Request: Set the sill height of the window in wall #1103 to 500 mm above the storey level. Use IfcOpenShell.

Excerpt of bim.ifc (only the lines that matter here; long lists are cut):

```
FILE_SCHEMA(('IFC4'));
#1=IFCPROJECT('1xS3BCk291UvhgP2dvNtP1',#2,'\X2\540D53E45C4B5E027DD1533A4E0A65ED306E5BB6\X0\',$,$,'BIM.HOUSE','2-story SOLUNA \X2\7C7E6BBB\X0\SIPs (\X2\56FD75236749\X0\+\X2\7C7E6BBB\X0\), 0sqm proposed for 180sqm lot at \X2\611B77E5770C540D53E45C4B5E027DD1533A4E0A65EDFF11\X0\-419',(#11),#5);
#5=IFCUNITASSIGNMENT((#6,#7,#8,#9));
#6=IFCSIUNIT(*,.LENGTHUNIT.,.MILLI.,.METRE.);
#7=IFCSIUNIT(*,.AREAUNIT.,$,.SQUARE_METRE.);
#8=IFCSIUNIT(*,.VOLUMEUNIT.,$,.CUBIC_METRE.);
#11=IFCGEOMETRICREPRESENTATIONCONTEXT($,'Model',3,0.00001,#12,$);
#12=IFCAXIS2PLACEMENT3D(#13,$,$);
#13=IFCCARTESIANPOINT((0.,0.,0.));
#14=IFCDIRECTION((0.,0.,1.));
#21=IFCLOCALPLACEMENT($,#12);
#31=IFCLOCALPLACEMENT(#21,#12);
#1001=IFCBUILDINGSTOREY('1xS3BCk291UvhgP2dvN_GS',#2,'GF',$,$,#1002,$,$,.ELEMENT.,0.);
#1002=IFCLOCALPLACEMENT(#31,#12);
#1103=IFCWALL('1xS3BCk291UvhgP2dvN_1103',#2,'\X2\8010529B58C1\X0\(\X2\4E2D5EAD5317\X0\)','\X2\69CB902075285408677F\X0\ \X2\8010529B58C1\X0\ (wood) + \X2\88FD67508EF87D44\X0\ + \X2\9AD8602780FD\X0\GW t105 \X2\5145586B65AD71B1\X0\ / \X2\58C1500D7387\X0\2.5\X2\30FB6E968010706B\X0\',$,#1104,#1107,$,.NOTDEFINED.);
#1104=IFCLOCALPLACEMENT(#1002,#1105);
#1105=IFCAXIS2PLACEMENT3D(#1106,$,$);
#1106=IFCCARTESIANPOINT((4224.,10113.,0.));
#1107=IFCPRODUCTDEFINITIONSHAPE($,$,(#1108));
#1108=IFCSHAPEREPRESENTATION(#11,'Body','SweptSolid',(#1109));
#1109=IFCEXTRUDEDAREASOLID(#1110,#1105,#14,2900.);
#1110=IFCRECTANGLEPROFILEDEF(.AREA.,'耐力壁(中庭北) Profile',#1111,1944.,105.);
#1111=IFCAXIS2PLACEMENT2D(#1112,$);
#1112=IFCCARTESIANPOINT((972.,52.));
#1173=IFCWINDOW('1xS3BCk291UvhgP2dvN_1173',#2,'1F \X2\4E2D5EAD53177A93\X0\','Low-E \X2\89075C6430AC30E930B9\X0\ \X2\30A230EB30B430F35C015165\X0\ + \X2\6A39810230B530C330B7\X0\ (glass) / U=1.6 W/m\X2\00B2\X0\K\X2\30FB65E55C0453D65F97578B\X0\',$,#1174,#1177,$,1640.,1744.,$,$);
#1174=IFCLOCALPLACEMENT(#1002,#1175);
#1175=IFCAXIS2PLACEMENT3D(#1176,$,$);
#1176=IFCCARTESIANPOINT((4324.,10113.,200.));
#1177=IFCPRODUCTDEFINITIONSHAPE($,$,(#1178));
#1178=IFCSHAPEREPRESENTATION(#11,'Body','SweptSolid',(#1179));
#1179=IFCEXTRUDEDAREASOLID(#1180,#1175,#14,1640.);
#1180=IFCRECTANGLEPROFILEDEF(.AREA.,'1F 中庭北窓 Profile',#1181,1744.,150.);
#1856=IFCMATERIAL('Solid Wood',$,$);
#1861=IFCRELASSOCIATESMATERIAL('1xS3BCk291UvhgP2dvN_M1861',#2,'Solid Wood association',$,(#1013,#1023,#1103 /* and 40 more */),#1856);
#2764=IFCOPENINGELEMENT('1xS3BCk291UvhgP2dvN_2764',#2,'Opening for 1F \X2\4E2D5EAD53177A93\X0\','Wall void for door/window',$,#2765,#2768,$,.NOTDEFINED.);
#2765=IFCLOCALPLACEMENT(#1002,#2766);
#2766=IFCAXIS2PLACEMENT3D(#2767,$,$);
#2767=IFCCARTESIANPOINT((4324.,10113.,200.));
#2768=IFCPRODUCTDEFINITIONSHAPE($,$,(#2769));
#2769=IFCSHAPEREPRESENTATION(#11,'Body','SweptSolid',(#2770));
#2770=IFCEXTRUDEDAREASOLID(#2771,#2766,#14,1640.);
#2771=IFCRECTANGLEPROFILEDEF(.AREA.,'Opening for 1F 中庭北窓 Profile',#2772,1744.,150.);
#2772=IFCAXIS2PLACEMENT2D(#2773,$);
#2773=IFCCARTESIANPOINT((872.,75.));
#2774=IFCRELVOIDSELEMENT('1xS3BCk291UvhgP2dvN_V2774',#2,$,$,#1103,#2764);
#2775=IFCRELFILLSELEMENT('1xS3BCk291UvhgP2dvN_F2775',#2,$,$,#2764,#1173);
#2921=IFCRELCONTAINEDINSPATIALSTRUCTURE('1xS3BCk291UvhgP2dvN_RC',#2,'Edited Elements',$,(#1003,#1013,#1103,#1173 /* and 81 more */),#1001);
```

```python
import numpy as np
import ifcopenshell
import ifcopenshell.api.geometry
import ifcopenshell.geom
import ifcopenshell.util.element
import ifcopenshell.util.placement
import ifcopenshell.util.shape
import ifcopenshell.util.unit

model = ifcopenshell.open("bim.ifc")
unit_scale = ifcopenshell.util.unit.calculate_unit_scale(model)

window = model.by_guid("1xS3BCk291UvhgP2dvN_1173")
opening = window.FillsVoids[0].RelatingOpeningElement
storey = ifcopenshell.util.element.get_container(window, ifc_class="IfcBuildingStorey")
level = ifcopenshell.util.placement.get_local_placement(storey.ObjectPlacement)[2, 3]

# The opening's origin need not be at the sill, so measure its lowest point.
shape = ifcopenshell.geom.create_shape(ifcopenshell.geom.settings(), opening)
bottom = ifcopenshell.util.shape.get_shape_bottom_elevation(shape, shape.geometry) / unit_scale
dz = level + 0.5 / unit_scale - bottom

shift = np.array([0.0, 0.0, dz])
# The window is not placed relative to its opening, so move both.
for product in (opening, window):
    matrix = ifcopenshell.util.placement.get_local_placement(product.ObjectPlacement)
    matrix[:3, 3] += shift
    ifcopenshell.api.geometry.edit_object_placement(model, product=product, matrix=matrix, is_si=False)

print(f"moved by {dz * unit_scale:+.3f} m")

model.write("bim_updated.ifc")
```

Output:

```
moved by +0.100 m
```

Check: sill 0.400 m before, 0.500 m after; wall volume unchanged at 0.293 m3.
